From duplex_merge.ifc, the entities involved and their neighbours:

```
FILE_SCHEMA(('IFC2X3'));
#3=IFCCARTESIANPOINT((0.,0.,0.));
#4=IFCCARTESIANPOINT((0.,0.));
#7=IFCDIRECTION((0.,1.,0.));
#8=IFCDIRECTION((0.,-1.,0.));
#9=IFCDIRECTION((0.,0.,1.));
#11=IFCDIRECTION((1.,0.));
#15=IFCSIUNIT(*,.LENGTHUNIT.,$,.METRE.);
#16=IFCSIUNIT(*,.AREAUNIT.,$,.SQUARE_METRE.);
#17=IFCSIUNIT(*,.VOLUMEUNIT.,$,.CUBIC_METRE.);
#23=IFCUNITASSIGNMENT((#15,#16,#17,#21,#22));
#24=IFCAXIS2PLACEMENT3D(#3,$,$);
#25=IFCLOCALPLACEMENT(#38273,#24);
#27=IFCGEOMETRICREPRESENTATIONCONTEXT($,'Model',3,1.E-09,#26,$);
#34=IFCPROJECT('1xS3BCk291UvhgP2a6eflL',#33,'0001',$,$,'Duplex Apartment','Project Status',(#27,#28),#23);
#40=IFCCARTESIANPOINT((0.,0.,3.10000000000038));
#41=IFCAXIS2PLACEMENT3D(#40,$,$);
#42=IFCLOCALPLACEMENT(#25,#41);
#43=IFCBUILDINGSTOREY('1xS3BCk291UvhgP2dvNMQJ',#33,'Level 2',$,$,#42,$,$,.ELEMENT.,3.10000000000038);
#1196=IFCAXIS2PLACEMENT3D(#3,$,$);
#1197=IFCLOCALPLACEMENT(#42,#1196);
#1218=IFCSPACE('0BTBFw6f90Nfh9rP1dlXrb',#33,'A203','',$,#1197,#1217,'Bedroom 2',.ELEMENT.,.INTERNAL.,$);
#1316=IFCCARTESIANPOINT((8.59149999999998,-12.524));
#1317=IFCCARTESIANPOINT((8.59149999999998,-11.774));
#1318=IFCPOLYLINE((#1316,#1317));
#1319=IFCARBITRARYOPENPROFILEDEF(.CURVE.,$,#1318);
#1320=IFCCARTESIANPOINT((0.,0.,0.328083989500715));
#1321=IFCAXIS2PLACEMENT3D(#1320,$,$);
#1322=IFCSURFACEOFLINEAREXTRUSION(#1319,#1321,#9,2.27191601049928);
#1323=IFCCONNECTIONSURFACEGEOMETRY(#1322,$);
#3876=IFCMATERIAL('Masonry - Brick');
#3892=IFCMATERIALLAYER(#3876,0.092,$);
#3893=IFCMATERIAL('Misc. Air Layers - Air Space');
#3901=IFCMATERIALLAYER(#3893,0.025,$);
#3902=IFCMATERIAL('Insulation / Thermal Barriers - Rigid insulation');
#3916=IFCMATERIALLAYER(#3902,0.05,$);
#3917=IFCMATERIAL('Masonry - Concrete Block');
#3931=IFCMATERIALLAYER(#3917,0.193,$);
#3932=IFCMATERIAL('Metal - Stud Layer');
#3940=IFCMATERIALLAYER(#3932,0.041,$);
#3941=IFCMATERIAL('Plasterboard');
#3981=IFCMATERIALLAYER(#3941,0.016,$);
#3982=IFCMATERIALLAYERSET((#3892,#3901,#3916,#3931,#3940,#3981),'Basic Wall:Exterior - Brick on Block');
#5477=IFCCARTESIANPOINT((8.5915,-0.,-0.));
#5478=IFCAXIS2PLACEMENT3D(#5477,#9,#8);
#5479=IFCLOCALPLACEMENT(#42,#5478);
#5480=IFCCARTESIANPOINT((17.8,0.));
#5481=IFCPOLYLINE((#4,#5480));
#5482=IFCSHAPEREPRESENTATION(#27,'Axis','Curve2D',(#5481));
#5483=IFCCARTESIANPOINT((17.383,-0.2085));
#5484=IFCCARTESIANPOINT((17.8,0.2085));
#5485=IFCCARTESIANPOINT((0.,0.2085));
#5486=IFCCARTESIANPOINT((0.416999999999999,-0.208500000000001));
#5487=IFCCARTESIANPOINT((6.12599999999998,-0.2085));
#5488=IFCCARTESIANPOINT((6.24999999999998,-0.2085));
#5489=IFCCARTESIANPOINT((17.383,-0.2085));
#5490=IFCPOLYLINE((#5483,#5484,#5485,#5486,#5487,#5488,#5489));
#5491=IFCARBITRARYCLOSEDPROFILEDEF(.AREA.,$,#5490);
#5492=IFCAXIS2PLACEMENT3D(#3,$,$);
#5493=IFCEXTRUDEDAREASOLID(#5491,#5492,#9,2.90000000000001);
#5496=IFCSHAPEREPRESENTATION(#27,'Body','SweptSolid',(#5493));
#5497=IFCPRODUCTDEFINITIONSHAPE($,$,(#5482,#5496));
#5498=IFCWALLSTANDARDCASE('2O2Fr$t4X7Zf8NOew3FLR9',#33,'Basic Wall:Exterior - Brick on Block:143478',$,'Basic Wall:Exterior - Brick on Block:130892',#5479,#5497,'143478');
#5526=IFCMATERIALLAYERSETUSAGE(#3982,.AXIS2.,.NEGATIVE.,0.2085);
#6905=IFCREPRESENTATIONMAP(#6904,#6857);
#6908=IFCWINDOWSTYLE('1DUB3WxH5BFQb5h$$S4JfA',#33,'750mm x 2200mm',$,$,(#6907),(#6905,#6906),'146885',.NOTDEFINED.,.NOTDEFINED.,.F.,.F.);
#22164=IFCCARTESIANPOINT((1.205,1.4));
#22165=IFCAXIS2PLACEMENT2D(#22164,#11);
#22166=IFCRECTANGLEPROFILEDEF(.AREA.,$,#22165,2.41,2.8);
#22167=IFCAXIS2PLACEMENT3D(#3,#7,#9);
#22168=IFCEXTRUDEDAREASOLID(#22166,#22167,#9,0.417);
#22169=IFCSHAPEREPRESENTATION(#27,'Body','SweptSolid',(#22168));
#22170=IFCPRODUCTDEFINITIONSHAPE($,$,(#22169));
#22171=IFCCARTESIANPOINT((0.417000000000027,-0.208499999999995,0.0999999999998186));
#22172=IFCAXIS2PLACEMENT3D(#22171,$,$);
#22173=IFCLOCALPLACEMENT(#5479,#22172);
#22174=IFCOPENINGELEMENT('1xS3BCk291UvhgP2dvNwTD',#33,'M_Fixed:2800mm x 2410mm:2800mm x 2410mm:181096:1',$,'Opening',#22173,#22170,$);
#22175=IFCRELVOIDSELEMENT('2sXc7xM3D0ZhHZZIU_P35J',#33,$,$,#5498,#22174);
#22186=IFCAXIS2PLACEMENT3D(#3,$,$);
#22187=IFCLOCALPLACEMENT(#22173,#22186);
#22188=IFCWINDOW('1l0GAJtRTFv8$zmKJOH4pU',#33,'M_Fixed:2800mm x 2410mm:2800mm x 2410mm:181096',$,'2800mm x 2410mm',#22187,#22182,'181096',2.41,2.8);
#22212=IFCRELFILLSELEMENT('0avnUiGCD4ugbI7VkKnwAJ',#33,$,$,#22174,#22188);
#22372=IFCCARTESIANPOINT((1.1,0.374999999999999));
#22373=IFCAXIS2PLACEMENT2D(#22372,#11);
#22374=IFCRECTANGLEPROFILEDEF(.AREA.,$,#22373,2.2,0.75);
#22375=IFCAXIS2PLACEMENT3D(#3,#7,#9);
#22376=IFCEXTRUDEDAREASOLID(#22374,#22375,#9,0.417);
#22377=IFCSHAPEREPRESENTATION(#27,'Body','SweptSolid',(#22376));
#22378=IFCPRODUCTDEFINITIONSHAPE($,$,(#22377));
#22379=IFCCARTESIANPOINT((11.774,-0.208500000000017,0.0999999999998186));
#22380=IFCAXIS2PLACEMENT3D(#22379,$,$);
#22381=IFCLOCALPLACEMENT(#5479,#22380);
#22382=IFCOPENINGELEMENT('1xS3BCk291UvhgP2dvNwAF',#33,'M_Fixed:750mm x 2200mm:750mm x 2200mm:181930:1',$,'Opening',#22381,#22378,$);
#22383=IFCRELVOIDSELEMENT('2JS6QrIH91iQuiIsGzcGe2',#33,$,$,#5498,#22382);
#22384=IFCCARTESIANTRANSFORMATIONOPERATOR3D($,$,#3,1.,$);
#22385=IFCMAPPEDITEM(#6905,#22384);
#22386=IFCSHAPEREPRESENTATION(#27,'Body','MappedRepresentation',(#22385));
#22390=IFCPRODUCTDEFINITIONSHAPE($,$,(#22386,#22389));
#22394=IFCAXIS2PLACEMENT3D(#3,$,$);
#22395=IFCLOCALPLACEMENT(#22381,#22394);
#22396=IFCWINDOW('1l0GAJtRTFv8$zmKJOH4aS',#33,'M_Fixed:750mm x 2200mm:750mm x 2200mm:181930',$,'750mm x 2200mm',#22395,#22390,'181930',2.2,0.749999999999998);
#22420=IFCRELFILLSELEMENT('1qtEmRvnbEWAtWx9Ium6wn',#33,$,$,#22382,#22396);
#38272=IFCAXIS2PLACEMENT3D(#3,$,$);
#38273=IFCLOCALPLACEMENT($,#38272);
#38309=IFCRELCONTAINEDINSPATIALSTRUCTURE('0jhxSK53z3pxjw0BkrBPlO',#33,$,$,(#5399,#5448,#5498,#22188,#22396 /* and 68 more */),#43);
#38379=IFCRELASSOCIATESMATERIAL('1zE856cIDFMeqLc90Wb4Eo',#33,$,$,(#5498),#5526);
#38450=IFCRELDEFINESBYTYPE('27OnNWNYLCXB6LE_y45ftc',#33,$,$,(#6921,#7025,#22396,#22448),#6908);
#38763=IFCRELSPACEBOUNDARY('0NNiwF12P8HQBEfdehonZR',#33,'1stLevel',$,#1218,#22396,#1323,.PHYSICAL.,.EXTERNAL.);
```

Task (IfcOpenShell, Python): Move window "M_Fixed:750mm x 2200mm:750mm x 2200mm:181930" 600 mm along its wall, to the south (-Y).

```python
import numpy as np
import ifcopenshell
import ifcopenshell.api.geometry
import ifcopenshell.util.placement
import ifcopenshell.util.unit

model = ifcopenshell.open("duplex_merge.ifc")
unit_scale = ifcopenshell.util.unit.calculate_unit_scale(model)

window = model.by_id(22396)
opening = window.FillsVoids[0].RelatingOpeningElement
wall = opening.VoidsElements[0].RelatingBuildingElement

wall_matrix = ifcopenshell.util.placement.get_local_placement(wall.ObjectPlacement)
shift = wall_matrix[:3, 0] * 0.6 / unit_scale
before = ifcopenshell.util.placement.get_local_placement(window.ObjectPlacement)[:3, 3].copy()

# The window is placed relative to its opening, so it follows when the opening moves.
matrix = ifcopenshell.util.placement.get_local_placement(opening.ObjectPlacement)
matrix[:3, 3] += shift
ifcopenshell.api.geometry.edit_object_placement(
    model, product=opening, matrix=matrix, is_si=False, should_transform_children=True
)

# Space boundary surfaces are stored in each space's coordinates; move them too.
for rel in window.ProvidesBoundaries:
    if not rel.ConnectionGeometry:
        continue
    surface = rel.ConnectionGeometry.SurfaceOnRelatingElement
    space_matrix = ifcopenshell.util.placement.get_local_placement(rel.RelatingSpace.ObjectPlacement)
    point = np.array(surface.Position.Location.Coordinates) + space_matrix[:3, :3].T @ shift
    surface.Position = model.createIfcAxis2Placement3D(
        model.createIfcCartesianPoint(point.tolist()), surface.Position.Axis, surface.Position.RefDirection
    )

after = ifcopenshell.util.placement.get_local_placement(window.ObjectPlacement)[:3, 3]
print("window moved by", (after - before).round(3) + 0.0)

model.write("duplex_merge_v2.ifc")
```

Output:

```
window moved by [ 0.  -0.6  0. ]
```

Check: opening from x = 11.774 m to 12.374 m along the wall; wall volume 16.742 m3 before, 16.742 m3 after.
